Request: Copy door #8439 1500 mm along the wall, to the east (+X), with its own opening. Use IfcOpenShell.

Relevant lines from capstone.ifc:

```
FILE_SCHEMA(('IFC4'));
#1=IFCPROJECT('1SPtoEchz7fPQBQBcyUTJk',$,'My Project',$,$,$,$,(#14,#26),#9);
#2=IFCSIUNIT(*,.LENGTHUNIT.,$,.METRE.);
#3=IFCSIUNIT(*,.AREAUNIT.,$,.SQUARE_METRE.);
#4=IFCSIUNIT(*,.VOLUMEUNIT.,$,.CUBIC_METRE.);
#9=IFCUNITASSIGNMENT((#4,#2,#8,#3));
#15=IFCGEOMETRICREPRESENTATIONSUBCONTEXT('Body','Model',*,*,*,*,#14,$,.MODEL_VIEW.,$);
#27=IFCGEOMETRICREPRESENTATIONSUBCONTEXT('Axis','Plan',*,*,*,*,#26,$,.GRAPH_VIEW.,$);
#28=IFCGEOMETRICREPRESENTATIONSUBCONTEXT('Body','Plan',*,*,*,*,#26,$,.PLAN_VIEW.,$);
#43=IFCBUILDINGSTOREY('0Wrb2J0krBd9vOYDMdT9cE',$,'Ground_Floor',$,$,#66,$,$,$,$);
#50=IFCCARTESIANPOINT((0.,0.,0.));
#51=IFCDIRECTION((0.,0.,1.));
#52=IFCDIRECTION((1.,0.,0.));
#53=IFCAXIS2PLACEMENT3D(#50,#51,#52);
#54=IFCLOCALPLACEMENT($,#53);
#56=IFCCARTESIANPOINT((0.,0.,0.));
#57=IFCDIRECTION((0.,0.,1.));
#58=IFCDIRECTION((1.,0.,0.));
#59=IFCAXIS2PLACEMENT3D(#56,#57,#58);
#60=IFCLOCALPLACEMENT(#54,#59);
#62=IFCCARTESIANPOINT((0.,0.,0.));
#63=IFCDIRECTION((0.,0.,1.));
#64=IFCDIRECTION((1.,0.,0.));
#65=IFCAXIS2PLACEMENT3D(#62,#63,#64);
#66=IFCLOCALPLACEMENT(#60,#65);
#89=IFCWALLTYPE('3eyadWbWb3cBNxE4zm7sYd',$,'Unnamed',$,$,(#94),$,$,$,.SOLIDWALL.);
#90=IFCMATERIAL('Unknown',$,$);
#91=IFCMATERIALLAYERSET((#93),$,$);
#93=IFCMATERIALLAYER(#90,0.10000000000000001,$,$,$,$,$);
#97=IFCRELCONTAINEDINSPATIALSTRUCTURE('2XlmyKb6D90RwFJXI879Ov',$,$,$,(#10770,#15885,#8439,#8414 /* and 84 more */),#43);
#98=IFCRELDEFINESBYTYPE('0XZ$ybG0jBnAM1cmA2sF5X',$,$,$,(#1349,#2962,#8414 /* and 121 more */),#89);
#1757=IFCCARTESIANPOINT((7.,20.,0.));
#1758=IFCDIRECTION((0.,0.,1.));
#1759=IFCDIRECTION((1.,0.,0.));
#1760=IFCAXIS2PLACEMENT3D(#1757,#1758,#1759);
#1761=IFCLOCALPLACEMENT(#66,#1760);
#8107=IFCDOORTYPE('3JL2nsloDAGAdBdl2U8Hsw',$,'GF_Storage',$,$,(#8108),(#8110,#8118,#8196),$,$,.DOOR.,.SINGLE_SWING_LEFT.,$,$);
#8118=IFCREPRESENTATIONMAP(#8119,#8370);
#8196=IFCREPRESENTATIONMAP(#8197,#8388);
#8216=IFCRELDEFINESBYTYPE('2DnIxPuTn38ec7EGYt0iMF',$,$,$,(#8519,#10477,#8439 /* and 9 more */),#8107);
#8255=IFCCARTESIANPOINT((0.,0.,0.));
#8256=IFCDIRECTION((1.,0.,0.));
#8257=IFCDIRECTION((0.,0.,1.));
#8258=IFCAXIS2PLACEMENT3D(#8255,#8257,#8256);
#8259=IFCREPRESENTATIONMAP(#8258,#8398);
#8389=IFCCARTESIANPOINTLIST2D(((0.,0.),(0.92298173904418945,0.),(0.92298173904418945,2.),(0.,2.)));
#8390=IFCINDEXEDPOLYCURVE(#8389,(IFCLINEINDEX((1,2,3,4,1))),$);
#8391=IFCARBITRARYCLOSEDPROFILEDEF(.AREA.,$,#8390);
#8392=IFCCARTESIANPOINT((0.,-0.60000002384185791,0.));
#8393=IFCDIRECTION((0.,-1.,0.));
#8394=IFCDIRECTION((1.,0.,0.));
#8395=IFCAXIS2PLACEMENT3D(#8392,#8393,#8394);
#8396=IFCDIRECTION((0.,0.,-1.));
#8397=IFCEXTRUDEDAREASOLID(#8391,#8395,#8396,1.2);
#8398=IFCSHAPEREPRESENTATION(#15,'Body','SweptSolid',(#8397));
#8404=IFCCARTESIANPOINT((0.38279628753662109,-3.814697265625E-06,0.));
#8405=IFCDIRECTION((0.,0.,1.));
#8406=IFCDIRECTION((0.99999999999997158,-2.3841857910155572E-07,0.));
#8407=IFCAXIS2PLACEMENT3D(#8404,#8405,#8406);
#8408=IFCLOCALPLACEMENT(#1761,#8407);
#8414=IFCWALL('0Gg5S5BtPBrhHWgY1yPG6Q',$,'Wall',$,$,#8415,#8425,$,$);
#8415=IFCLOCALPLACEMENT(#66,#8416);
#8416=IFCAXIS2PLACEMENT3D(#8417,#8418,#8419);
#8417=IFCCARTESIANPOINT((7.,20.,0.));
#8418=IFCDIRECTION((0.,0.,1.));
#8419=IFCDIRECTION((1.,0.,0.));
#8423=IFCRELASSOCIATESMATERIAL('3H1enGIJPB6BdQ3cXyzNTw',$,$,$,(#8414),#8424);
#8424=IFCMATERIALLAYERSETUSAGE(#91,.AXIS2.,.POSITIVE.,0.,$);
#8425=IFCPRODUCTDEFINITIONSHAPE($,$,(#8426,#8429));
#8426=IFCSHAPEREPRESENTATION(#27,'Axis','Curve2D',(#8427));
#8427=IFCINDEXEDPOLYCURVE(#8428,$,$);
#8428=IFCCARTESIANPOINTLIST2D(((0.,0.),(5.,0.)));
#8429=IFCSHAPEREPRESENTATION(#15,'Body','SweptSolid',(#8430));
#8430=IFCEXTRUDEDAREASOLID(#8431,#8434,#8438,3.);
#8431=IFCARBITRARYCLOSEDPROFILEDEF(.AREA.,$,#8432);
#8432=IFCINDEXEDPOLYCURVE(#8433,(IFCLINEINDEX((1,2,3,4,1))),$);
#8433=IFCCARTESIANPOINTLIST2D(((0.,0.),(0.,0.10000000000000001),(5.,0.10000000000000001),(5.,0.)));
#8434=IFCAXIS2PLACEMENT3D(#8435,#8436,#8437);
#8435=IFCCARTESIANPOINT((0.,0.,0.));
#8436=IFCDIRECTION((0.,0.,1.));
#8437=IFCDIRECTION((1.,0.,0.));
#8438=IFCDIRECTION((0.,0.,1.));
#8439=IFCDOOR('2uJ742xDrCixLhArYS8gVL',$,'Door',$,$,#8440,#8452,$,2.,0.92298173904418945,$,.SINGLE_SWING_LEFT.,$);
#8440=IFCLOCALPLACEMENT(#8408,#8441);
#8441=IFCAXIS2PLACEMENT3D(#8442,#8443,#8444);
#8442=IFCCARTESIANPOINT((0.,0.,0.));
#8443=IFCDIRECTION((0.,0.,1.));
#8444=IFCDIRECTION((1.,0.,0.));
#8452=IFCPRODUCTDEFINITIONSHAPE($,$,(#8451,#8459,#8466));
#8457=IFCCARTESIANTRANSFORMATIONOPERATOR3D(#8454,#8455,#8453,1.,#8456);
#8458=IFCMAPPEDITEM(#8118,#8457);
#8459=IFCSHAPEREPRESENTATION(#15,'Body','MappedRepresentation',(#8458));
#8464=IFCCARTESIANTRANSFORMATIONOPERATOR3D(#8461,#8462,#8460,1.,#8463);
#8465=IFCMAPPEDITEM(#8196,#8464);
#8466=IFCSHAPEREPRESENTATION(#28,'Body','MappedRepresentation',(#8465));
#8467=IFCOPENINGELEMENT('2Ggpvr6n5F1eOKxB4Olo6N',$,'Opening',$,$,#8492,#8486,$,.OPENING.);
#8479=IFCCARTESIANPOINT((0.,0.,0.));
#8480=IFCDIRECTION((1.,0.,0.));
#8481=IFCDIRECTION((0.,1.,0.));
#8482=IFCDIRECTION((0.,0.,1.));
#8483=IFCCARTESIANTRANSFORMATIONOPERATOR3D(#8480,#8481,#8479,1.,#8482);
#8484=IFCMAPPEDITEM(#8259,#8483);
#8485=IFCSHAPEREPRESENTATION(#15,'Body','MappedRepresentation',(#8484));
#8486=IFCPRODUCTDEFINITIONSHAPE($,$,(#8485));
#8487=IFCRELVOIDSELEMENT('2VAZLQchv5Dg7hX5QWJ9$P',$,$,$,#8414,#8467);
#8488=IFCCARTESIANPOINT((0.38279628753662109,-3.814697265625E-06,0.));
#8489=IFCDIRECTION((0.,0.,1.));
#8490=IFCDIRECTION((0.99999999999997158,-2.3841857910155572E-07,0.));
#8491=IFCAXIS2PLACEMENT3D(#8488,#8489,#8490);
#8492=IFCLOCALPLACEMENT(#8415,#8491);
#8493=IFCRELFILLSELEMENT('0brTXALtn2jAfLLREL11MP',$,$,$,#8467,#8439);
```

```python
import ifcopenshell
import ifcopenshell.api.feature
import ifcopenshell.api.geometry
import ifcopenshell.api.root
import ifcopenshell.geom
import ifcopenshell.util.element
import ifcopenshell.util.placement
import ifcopenshell.util.shape
import ifcopenshell.util.unit

model = ifcopenshell.open("capstone.ifc")
unit_scale = ifcopenshell.util.unit.calculate_unit_scale(model)
settings = ifcopenshell.geom.settings()


def volume(element):
    """Net volume in cubic metres, openings subtracted."""
    shape = ifcopenshell.geom.create_shape(settings, element)
    return ifcopenshell.util.shape.get_volume(shape.geometry)


door = model.by_guid("2uJ742xDrCixLhArYS8gVL")
opening = door.FillsVoids[0].RelatingOpeningElement
wall = opening.VoidsElements[0].RelatingBuildingElement
before = volume(wall)
shift = ifcopenshell.util.placement.get_local_placement(wall.ObjectPlacement)[:3, 0] * 1.5 / unit_scale

# copy_class copies the void relationship, type, container and properties, but no geometry.
new_opening = ifcopenshell.api.root.copy_class(model, product=opening)
new_opening.Representation = ifcopenshell.util.element.copy_deep(
    model, opening.Representation, exclude=["IfcGeometricRepresentationContext", "IfcRepresentationMap"]
)
new_door = ifcopenshell.api.root.copy_class(model, product=door)
new_door.Representation = ifcopenshell.util.element.copy_deep(
    model, door.Representation, exclude=["IfcGeometricRepresentationContext", "IfcRepresentationMap"]
)
ifcopenshell.api.feature.add_filling(model, opening=new_opening, element=new_door)

for old, new in ((opening, new_opening), (door, new_door)):
    matrix = ifcopenshell.util.placement.get_local_placement(old.ObjectPlacement)
    matrix[:3, 3] += shift
    ifcopenshell.api.geometry.edit_object_placement(model, product=new, matrix=matrix, is_si=False)

after = volume(wall)

print(f"wall volume {before:.3f} -> {after:.3f} m3")

model.write("capstone-out.ifc")
```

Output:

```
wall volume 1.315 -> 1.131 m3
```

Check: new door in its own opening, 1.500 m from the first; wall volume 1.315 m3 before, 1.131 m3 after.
